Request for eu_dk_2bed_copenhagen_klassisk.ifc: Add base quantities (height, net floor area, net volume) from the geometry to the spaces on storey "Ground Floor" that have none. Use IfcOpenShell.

First a look at what the model holds.

```python
import ifcopenshell
import ifcopenshell.util.element
import ifcopenshell.util.unit

model = ifcopenshell.open("eu_dk_2bed_copenhagen_klassisk.ifc")
print(model.schema)
for unit_type in ("LENGTHUNIT", "AREAUNIT", "VOLUMEUNIT"):
    print(unit_type, ifcopenshell.util.unit.calculate_unit_scale(model, unit_type))
storey = next(s for s in model.by_type("IfcBuildingStorey") if s.Name == "Ground Floor")
spaces = [e for e in ifcopenshell.util.element.get_decomposition(storey) if e.is_a("IfcSpace")]
for e in sorted(spaces, key=lambda e: e.id()):
    print(e.id(), e.is_a(), e.Name, list(ifcopenshell.util.element.get_psets(e, qtos_only=True)), sep=" | ")
```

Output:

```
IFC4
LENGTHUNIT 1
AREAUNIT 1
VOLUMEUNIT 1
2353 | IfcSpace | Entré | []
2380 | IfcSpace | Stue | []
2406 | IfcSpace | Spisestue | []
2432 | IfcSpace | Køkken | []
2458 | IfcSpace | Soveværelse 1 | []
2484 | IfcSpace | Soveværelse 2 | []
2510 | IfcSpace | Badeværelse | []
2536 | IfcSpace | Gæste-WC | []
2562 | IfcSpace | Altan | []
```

```python
import ifcopenshell
import ifcopenshell.api.pset
import ifcopenshell.geom
import ifcopenshell.util.element
import ifcopenshell.util.shape
import ifcopenshell.util.unit

model = ifcopenshell.open("eu_dk_2bed_copenhagen_klassisk.ifc")
unit_scale = ifcopenshell.util.unit.calculate_unit_scale(model)
area_scale = ifcopenshell.util.unit.calculate_unit_scale(model, "AREAUNIT")
volume_scale = ifcopenshell.util.unit.calculate_unit_scale(model, "VOLUMEUNIT")
settings = ifcopenshell.geom.settings()

storey = next(s for s in model.by_type("IfcBuildingStorey") if s.Name == "Ground Floor")
spaces = [e for e in ifcopenshell.util.element.get_decomposition(storey) if e.is_a("IfcSpace")]

for e in sorted(spaces, key=lambda e: e.id()):
    if ifcopenshell.util.element.get_psets(e, qtos_only=True, should_inherit=False):
        continue
    # Geometry comes back in metres, in the element's own axes.
    shape = ifcopenshell.geom.create_shape(settings, e)
    values = {
        "Height": ifcopenshell.util.shape.get_z(shape.geometry) / unit_scale,
        "NetFloorArea": ifcopenshell.util.shape.get_footprint_area(shape.geometry) / area_scale,
        "NetVolume": ifcopenshell.util.shape.get_volume(shape.geometry) / volume_scale,
    }
    qto = ifcopenshell.api.pset.add_qto(model, product=e, name="Qto_SpaceBaseQuantities")
    ifcopenshell.api.pset.edit_qto(model, qto=qto, properties=values)
    print(e.id(), {k: round(v, 3) for k, v in values.items()})

model.write("eu_dk_2bed_copenhagen_klassisk_v2.ifc")
```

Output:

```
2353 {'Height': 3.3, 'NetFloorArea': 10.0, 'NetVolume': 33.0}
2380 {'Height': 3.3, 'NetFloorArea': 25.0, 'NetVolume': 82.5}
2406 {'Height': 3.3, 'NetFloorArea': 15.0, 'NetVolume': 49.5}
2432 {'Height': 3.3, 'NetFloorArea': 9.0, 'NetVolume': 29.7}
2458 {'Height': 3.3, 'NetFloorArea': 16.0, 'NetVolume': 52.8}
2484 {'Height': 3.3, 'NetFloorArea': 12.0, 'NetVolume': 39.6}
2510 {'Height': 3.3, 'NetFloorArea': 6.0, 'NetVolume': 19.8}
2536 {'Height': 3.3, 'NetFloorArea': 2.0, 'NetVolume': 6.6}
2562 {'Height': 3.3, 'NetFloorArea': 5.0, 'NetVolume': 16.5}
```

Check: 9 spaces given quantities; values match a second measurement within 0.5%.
